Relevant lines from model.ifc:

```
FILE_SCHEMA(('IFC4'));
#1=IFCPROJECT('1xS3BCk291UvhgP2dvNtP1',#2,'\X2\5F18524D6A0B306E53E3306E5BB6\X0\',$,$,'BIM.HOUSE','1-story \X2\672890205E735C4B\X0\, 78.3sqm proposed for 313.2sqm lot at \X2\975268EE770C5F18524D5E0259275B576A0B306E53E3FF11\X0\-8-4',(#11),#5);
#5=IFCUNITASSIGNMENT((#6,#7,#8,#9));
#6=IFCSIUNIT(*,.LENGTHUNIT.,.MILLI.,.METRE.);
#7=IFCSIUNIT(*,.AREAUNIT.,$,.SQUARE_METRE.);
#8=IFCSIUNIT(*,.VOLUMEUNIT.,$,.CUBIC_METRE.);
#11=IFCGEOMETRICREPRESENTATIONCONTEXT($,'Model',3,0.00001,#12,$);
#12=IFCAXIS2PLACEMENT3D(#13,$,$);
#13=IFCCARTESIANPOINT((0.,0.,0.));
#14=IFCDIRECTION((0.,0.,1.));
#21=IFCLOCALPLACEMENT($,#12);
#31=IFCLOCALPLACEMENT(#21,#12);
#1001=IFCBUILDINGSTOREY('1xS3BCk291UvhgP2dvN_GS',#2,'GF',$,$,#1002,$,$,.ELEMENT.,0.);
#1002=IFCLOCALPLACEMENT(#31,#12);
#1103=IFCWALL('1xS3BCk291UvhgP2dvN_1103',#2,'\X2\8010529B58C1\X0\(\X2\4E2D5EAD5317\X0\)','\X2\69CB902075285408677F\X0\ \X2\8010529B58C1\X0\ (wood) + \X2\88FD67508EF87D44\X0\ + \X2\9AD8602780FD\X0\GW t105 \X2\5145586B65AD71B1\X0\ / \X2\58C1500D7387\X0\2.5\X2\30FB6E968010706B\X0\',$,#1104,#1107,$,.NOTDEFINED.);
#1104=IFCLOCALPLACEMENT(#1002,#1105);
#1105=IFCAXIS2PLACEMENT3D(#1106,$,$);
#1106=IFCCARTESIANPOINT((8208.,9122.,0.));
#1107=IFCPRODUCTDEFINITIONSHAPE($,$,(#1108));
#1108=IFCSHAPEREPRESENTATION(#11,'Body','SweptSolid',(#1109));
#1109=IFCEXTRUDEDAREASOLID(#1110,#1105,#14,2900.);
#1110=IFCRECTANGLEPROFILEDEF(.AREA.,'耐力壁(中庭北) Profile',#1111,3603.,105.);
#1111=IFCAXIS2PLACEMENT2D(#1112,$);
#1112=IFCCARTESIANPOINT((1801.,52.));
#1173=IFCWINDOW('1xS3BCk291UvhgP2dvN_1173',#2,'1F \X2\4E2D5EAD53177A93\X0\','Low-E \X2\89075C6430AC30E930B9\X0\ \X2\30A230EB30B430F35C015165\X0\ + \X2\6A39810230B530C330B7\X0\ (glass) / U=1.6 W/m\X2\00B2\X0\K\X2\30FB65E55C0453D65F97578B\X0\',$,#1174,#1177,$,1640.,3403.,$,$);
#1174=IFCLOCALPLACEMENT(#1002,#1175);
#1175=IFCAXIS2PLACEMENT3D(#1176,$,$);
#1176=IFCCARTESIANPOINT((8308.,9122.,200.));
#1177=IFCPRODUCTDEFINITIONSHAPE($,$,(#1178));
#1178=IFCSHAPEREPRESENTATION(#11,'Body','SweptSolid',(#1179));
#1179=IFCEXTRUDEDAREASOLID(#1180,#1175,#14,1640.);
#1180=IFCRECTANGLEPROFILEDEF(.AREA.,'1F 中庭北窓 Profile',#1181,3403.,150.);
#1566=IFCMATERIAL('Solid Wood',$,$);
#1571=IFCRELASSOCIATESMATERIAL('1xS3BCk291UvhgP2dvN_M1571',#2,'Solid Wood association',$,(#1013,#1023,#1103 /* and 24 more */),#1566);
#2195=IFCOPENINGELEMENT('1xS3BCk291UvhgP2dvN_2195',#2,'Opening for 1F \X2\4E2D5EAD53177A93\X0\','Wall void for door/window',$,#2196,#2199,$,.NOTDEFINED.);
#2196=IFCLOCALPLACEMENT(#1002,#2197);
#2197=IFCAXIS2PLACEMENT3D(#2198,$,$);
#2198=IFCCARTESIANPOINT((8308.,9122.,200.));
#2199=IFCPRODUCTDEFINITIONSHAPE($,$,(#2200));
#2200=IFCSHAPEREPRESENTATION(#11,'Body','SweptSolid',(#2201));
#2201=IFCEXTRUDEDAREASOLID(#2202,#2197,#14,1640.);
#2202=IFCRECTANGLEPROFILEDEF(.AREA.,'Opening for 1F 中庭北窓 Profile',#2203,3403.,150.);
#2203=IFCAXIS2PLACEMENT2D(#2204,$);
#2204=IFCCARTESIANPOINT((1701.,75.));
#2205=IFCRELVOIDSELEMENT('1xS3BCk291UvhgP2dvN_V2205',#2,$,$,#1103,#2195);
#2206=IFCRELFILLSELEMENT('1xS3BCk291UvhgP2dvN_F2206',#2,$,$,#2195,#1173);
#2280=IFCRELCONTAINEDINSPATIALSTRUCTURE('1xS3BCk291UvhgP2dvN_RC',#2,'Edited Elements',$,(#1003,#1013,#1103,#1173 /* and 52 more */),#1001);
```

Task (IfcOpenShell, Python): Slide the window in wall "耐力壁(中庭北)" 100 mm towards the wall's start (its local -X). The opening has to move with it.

```python
import ifcopenshell
import ifcopenshell.api.geometry
import ifcopenshell.util.placement

model = ifcopenshell.open("model.ifc")

window = model.by_id(1173)
opening = window.FillsVoids[0].RelatingOpeningElement
wall = opening.VoidsElements[0].RelatingBuildingElement

wall_matrix = ifcopenshell.util.placement.get_local_placement(wall.ObjectPlacement)
shift = wall_matrix[:3, 0] * -100.0
before = ifcopenshell.util.placement.get_local_placement(window.ObjectPlacement)[:3, 3].copy()

# The window is not placed relative to its opening, so move both.
for product in (opening, window):
    matrix = ifcopenshell.util.placement.get_local_placement(product.ObjectPlacement)
    matrix[:3, 3] += shift
    ifcopenshell.api.geometry.edit_object_placement(model, product=product, matrix=matrix, is_si=False)

after = ifcopenshell.util.placement.get_local_placement(window.ObjectPlacement)[:3, 3]
print("window moved by", (after - before).round(3) + 0.0)

model.write("model_v2.ifc")
```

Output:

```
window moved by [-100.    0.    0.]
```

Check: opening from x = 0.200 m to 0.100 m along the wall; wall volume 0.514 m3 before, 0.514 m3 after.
